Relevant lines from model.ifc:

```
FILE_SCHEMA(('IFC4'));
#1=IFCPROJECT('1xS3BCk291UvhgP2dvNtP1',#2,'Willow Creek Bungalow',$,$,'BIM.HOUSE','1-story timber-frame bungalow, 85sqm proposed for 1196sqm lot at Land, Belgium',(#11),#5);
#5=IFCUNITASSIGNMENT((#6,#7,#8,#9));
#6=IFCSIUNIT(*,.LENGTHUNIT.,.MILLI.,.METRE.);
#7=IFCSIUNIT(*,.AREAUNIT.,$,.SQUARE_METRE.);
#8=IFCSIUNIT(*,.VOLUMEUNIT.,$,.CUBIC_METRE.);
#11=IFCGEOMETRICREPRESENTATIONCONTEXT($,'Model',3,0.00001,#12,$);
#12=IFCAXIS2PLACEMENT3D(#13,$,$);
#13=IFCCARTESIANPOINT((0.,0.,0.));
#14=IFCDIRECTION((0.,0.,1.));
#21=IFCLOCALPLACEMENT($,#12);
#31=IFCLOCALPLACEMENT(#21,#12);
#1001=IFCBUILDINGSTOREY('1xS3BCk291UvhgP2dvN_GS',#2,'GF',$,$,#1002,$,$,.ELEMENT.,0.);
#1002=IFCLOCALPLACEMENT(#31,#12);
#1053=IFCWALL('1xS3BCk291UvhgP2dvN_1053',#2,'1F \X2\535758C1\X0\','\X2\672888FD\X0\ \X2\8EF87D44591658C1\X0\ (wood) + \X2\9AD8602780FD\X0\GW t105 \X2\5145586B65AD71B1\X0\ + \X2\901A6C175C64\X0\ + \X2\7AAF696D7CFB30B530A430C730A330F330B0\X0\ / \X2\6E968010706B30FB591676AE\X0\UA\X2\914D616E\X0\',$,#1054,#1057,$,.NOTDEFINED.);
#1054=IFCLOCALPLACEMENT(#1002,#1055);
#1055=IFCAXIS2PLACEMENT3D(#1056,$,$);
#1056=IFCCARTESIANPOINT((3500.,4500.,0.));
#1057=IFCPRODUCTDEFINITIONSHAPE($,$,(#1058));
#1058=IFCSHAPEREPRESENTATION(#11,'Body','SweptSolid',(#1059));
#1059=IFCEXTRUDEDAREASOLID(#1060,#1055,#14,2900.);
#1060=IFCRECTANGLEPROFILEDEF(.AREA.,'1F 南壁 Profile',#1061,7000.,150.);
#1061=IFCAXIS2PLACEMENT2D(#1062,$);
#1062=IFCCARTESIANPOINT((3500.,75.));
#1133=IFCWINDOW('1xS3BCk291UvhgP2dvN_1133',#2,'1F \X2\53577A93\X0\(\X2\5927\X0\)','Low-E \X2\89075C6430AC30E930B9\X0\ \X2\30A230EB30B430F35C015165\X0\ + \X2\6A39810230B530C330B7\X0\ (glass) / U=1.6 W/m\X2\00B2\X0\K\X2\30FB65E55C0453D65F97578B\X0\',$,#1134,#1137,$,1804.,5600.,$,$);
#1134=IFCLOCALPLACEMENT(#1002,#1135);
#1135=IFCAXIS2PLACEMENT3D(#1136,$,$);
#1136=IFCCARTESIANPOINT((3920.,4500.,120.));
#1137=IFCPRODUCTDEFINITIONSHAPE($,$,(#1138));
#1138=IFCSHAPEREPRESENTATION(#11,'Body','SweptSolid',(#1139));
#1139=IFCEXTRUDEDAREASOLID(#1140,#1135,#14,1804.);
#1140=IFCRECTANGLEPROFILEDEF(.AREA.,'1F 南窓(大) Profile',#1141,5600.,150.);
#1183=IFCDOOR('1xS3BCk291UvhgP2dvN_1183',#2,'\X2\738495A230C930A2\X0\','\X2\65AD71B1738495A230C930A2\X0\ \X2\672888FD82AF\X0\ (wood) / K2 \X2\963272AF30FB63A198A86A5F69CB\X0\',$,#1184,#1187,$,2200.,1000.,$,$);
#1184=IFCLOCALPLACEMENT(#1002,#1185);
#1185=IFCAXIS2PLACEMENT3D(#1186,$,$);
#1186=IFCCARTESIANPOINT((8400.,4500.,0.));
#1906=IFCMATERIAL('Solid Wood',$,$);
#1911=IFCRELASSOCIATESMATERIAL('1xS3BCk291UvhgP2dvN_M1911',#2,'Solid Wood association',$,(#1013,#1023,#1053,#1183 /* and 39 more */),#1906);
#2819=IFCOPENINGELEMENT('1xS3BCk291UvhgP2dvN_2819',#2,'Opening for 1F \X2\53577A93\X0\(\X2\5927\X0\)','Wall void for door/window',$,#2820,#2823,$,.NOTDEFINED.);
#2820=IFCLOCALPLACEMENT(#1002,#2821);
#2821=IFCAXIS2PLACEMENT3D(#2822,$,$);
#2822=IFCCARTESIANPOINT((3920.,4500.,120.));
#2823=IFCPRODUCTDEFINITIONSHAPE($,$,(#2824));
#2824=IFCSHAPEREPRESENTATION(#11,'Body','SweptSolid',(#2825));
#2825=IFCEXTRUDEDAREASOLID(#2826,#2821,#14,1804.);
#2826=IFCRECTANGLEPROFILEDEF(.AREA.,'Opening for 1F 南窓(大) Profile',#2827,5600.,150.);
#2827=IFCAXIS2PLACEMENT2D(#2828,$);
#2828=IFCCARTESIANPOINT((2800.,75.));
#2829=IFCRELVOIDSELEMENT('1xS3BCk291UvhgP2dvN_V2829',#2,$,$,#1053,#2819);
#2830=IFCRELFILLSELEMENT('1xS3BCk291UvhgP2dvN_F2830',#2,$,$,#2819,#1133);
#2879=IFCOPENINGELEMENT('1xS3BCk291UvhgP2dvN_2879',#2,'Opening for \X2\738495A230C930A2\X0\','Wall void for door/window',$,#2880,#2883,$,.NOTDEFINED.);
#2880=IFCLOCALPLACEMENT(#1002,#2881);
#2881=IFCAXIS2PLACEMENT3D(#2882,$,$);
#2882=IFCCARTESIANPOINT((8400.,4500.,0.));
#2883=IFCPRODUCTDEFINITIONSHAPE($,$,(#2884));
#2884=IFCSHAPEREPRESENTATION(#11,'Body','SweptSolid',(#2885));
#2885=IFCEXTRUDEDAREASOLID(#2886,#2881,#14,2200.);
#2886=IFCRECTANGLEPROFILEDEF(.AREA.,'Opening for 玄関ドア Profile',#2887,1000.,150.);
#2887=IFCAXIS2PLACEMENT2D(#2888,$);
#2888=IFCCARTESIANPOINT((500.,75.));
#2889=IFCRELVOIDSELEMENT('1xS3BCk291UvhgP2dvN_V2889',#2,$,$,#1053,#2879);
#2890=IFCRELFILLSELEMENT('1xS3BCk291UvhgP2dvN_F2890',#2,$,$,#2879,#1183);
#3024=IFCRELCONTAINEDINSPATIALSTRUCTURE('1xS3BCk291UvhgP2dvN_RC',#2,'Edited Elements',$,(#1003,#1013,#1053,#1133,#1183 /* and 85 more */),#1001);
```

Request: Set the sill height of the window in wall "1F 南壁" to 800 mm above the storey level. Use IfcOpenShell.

```python
import numpy as np
import ifcopenshell
import ifcopenshell.api.geometry
import ifcopenshell.geom
import ifcopenshell.util.element
import ifcopenshell.util.placement
import ifcopenshell.util.shape
import ifcopenshell.util.unit

model = ifcopenshell.open("model.ifc")
unit_scale = ifcopenshell.util.unit.calculate_unit_scale(model)

window = model.by_id(1133)
opening = window.FillsVoids[0].RelatingOpeningElement
storey = ifcopenshell.util.element.get_container(window, ifc_class="IfcBuildingStorey")
level = ifcopenshell.util.placement.get_local_placement(storey.ObjectPlacement)[2, 3]

# The opening's origin need not be at the sill, so measure its lowest point.
shape = ifcopenshell.geom.create_shape(ifcopenshell.geom.settings(), opening)
bottom = ifcopenshell.util.shape.get_shape_bottom_elevation(shape, shape.geometry) / unit_scale
dz = level + 0.8 / unit_scale - bottom

shift = np.array([0.0, 0.0, dz])
# The window is not placed relative to its opening, so move both.
for product in (opening, window):
    matrix = ifcopenshell.util.placement.get_local_placement(product.ObjectPlacement)
    matrix[:3, 3] += shift
    ifcopenshell.api.geometry.edit_object_placement(model, product=product, matrix=matrix, is_si=False)

print(f"moved by {dz * unit_scale:+.3f} m")

model.write("model_edited.ifc")
```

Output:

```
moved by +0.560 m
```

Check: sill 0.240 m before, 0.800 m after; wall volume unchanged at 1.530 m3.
